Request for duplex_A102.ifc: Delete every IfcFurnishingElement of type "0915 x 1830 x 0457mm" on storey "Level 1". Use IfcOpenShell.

First a look at what the model holds.

```python
import ifcopenshell
import ifcopenshell.util.element

model = ifcopenshell.open("duplex_A102.ifc")
print(model.schema)
storey = next(s for s in model.by_type("IfcBuildingStorey") if s.Name == "Level 1")
furniture = [e for e in ifcopenshell.util.element.get_decomposition(storey) if e.is_a("IfcFurnishingElement")]
seen = {}
for e in furniture:
    element_type = ifcopenshell.util.element.get_type(e)
    name = element_type.Name if element_type not in (None, e) else None
    seen[name] = seen.get(name, 0) + 1
for name, count in sorted(seen.items(), key=str):
    print(count, "x", name)
```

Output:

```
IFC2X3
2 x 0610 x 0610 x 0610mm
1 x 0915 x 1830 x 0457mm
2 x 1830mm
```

```python
import ifcopenshell
import ifcopenshell.api.root
import ifcopenshell.util.element

model = ifcopenshell.open("duplex_A102.ifc")

storey = next(s for s in model.by_type("IfcBuildingStorey") if s.Name == "Level 1")
furniture = [e for e in ifcopenshell.util.element.get_decomposition(storey) if e.is_a("IfcFurnishingElement")]
targets = [e for e in furniture if (t := ifcopenshell.util.element.get_type(e)) not in (None, e) and t.Name == "0915 x 1830 x 0457mm"]

for e in targets:
    ifcopenshell.api.root.remove_product(model, product=e)
print(len(targets), "removed")

model.write("duplex_A102_rev.ifc")
```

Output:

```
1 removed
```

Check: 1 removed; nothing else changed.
